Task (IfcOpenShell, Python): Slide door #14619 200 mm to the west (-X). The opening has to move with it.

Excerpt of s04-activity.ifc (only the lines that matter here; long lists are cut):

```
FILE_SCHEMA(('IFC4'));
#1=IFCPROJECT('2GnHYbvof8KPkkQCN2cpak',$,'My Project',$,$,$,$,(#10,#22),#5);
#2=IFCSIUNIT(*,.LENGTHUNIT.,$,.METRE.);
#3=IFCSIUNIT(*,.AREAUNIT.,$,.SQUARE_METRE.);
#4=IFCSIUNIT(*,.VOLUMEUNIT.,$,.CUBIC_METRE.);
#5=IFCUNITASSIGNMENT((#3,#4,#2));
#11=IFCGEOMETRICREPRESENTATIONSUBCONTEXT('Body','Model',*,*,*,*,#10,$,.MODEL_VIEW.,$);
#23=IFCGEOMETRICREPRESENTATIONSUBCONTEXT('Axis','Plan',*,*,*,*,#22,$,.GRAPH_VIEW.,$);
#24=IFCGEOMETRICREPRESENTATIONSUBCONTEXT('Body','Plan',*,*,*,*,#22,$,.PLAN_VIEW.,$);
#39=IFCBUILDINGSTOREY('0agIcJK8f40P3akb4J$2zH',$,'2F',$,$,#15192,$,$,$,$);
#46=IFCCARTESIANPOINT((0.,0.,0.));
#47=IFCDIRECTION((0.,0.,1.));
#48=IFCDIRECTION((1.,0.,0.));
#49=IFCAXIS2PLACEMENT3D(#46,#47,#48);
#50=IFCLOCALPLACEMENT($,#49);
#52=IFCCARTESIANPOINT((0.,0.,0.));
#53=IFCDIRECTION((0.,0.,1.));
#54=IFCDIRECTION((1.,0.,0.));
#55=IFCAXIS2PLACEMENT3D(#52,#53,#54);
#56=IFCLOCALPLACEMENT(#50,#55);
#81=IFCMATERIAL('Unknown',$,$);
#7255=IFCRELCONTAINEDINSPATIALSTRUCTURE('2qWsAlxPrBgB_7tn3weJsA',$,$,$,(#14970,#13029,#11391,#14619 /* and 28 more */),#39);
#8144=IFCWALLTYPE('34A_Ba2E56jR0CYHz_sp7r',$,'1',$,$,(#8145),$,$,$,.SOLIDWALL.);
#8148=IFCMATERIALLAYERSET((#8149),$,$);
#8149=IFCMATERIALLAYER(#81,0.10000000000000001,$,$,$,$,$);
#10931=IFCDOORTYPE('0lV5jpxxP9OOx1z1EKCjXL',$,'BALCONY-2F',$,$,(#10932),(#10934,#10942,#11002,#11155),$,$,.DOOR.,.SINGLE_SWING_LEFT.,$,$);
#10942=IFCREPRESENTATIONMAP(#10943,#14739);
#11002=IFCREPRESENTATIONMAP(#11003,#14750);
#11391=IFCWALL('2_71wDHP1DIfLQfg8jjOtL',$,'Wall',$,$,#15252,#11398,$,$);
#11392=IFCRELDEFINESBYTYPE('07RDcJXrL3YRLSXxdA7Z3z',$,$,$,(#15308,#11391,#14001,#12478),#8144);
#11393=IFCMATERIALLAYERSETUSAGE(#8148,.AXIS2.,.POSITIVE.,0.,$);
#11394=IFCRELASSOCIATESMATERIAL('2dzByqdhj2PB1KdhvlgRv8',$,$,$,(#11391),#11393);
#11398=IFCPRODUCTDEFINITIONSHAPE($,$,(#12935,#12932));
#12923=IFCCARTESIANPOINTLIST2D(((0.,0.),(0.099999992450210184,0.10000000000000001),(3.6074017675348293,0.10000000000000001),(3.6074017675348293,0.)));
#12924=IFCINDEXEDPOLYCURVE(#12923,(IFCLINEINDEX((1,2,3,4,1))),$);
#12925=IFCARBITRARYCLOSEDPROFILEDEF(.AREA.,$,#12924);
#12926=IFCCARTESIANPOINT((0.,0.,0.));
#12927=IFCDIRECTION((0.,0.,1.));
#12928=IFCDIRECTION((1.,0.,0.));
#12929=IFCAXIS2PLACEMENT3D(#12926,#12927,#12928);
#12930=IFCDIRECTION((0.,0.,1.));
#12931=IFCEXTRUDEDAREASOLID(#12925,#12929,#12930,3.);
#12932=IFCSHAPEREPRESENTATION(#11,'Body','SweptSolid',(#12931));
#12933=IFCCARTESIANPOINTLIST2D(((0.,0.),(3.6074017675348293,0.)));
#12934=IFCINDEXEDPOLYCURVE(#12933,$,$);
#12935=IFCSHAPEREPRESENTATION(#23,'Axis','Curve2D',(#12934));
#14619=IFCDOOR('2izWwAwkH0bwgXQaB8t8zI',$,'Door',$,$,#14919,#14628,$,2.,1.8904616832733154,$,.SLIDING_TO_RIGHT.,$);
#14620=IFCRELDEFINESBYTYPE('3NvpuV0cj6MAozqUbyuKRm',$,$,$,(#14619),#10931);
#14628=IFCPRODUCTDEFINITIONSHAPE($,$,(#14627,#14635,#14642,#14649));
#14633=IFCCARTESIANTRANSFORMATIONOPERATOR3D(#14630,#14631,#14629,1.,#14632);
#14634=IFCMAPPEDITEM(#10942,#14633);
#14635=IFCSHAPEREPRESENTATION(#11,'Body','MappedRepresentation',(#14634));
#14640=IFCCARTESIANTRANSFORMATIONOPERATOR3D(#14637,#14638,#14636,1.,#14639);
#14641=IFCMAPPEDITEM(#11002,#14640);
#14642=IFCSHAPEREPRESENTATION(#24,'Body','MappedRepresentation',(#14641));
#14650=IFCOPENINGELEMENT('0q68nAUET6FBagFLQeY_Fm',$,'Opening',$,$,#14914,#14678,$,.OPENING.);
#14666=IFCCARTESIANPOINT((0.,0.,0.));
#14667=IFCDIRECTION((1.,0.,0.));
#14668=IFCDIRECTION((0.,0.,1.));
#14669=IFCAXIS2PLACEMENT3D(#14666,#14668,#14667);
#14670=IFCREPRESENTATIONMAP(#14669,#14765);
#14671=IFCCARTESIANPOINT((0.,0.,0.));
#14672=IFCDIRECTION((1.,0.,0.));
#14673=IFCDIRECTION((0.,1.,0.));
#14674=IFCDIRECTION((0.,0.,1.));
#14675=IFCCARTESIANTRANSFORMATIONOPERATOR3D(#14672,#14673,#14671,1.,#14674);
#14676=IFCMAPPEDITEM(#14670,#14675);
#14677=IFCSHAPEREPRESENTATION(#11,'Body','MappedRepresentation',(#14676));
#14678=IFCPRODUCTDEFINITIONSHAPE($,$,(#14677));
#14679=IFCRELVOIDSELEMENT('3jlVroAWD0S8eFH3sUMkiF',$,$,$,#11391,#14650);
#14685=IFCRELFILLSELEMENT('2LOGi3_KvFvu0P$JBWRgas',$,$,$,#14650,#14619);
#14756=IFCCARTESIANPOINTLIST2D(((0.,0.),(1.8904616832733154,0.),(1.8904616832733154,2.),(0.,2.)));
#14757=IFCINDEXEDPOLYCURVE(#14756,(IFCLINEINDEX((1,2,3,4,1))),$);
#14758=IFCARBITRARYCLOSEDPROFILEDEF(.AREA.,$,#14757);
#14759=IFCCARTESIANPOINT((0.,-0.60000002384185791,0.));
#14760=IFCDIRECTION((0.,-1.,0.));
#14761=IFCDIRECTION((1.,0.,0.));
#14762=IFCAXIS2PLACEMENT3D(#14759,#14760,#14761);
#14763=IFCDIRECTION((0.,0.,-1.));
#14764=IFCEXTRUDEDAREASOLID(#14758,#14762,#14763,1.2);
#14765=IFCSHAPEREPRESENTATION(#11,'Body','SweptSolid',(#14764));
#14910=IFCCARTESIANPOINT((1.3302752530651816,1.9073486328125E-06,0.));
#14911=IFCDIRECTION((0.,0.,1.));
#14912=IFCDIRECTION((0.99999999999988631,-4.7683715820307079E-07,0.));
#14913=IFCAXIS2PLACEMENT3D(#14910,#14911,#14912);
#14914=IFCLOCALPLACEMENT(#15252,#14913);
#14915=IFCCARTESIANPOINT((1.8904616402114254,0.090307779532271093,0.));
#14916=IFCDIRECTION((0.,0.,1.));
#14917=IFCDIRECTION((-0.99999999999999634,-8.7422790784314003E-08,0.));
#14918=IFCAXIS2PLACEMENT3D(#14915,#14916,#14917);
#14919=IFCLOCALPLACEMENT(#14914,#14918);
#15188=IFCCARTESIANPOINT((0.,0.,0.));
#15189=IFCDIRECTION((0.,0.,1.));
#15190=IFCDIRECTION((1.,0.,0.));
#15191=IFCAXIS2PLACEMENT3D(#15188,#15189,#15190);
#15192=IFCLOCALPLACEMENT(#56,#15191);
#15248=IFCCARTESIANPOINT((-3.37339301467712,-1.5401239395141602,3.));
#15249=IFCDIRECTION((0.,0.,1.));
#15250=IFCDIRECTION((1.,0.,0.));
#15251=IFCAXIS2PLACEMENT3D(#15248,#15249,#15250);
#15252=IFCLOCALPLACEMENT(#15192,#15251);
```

```python
import ifcopenshell
import ifcopenshell.api.geometry
import ifcopenshell.util.placement
import ifcopenshell.util.unit

model = ifcopenshell.open("s04-activity.ifc")
unit_scale = ifcopenshell.util.unit.calculate_unit_scale(model)

door = model.by_guid("2izWwAwkH0bwgXQaB8t8zI")
opening = door.FillsVoids[0].RelatingOpeningElement
wall = opening.VoidsElements[0].RelatingBuildingElement

wall_matrix = ifcopenshell.util.placement.get_local_placement(wall.ObjectPlacement)
shift = wall_matrix[:3, 0] * -0.2 / unit_scale
before = ifcopenshell.util.placement.get_local_placement(door.ObjectPlacement)[:3, 3].copy()

# The door is placed relative to its opening, so it follows when the opening moves.
matrix = ifcopenshell.util.placement.get_local_placement(opening.ObjectPlacement)
matrix[:3, 3] += shift
ifcopenshell.api.geometry.edit_object_placement(
    model, product=opening, matrix=matrix, is_si=False, should_transform_children=True
)

after = ifcopenshell.util.placement.get_local_placement(door.ObjectPlacement)[:3, 3]
print("door moved by", (after - before).round(3) + 0.0)

model.write("s04-activity_rev.ifc")
```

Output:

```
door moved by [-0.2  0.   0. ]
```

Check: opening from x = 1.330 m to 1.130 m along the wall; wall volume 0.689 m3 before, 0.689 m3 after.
